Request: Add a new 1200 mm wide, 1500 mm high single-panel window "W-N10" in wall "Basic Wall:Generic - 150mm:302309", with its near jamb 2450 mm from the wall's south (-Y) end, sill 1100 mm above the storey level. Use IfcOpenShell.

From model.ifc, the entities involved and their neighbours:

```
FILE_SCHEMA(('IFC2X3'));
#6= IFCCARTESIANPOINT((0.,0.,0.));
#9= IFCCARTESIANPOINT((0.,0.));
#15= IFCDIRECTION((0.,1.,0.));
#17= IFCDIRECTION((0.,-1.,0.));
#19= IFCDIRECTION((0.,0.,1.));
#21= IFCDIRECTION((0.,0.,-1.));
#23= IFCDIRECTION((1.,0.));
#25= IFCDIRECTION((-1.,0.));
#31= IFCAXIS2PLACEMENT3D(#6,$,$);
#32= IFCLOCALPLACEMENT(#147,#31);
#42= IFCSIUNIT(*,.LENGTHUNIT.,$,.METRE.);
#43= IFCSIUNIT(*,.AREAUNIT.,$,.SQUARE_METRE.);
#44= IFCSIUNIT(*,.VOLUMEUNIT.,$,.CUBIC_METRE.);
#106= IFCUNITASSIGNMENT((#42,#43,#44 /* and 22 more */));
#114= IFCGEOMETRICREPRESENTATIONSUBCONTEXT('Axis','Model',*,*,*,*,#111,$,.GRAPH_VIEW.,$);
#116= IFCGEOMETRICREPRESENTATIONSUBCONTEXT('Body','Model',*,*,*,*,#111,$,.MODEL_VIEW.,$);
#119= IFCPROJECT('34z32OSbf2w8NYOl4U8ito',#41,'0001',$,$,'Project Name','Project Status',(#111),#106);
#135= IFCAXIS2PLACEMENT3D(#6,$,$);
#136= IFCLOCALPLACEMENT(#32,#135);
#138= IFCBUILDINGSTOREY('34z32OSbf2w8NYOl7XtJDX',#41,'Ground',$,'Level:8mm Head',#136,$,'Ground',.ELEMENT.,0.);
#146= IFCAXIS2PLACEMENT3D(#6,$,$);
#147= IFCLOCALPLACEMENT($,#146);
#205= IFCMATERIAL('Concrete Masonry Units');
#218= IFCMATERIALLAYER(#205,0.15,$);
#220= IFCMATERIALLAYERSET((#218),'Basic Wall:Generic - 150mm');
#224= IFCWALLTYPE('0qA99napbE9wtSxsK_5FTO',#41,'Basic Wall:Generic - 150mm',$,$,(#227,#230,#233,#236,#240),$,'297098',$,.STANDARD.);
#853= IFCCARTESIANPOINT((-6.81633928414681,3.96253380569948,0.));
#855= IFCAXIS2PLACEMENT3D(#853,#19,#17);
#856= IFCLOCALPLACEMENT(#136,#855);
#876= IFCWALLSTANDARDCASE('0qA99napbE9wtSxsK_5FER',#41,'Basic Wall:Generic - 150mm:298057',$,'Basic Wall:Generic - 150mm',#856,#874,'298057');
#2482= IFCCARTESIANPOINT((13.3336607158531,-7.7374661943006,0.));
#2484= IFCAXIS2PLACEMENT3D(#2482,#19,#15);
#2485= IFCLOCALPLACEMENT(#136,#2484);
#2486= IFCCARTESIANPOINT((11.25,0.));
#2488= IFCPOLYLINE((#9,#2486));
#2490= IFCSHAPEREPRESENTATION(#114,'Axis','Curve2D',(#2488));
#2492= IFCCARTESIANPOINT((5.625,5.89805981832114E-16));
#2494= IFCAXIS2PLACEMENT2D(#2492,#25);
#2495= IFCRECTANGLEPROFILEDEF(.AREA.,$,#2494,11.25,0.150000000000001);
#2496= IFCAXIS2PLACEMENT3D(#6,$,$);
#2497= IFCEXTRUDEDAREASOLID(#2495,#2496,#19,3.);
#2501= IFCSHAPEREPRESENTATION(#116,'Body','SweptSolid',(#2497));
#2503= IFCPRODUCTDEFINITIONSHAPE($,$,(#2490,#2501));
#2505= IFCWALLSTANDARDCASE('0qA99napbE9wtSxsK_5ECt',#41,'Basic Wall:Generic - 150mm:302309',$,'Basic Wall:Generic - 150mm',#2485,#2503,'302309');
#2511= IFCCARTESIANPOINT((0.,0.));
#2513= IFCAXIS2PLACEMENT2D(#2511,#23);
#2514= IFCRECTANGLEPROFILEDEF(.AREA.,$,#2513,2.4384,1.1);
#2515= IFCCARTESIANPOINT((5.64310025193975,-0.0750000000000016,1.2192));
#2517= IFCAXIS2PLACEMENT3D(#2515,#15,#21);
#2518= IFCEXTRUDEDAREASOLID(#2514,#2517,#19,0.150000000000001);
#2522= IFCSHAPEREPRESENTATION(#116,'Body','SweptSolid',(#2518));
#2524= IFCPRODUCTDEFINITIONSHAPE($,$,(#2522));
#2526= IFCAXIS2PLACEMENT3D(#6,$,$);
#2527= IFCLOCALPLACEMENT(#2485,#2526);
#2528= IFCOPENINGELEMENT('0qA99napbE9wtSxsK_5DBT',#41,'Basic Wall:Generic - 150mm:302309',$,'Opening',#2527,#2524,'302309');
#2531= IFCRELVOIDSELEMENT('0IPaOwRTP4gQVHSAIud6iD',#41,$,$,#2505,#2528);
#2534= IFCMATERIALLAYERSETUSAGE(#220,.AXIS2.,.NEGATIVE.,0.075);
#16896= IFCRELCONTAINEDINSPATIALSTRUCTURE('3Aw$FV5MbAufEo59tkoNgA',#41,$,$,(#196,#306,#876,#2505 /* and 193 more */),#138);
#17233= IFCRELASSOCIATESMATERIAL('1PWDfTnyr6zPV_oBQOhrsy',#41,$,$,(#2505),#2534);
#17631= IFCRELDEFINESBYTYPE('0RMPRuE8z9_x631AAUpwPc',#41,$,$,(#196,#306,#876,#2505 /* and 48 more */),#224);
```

```python
import numpy as np
import ifcopenshell
import ifcopenshell.api.feature
import ifcopenshell.api.geometry
import ifcopenshell.api.root
import ifcopenshell.api.spatial
import ifcopenshell.api.type
import ifcopenshell.geom
import ifcopenshell.util.element
import ifcopenshell.util.placement
import ifcopenshell.util.representation
import ifcopenshell.util.shape
import ifcopenshell.util.unit

model = ifcopenshell.open("model.ifc")
unit_scale = ifcopenshell.util.unit.calculate_unit_scale(model)
settings = ifcopenshell.geom.settings()


def volume(element):
    """Net volume in cubic metres, openings subtracted."""
    shape = ifcopenshell.geom.create_shape(settings, element)
    return ifcopenshell.util.shape.get_volume(shape.geometry)


wall = model.by_guid("0qA99napbE9wtSxsK_5ECt")
storey = ifcopenshell.util.element.get_container(wall, ifc_class="IfcBuildingStorey")
context = ifcopenshell.util.representation.get_context(model, "Model", "Body", "MODEL_VIEW")
before = volume(wall)

width, height, from_end, sill = 1.2, 1.5, 2.45, 1.1  # metres

# The wall runs along its own X axis, and the end named is its -X end.
wall_shape = ifcopenshell.geom.create_shape(settings, wall)
x, y, z = ifcopenshell.util.shape.get_vertices(wall_shape.geometry).T
start = x.min() + from_end
face, thickness = float(y.min()), float(y.max() - y.min())
wall_matrix = ifcopenshell.util.placement.get_local_placement(wall.ObjectPlacement)
level = ifcopenshell.util.placement.get_local_placement(storey.ObjectPlacement)[2, 3]


def in_wall(x, y):
    """Placement at x, y metres in the wall's axes, at sill height."""
    matrix = wall_matrix.copy()
    matrix[:, 3] = wall_matrix @ np.array([x / unit_scale, y / unit_scale, 0.0, 1.0])
    matrix[2, 3] = level + sill / unit_scale
    return matrix


# Opening: a box that overshoots both wall faces by 50 mm.
opening = ifcopenshell.api.root.create_entity(model, ifc_class="IfcOpeningElement")
box = ifcopenshell.api.geometry.add_wall_representation(
    model, context=context, length=width, height=height, thickness=thickness + 0.1
)
ifcopenshell.api.geometry.assign_representation(model, product=opening, representation=box)
ifcopenshell.api.geometry.edit_object_placement(model, product=opening, matrix=in_wall(start, face - 0.05), is_si=False)
ifcopenshell.api.feature.add_feature(model, feature=opening, element=wall)

window = ifcopenshell.api.root.create_entity(model, ifc_class="IfcWindow", name="W-N10")
window.OverallWidth, window.OverallHeight = width / unit_scale, height / unit_scale
body = ifcopenshell.api.geometry.add_window_representation(
    model,
    context=context,
    overall_width=window.OverallWidth,
    overall_height=window.OverallHeight,
    partition_type="SINGLE_PANEL",
)
ifcopenshell.api.geometry.assign_representation(model, product=window, representation=body)
ifcopenshell.api.spatial.assign_container(model, products=[window], relating_structure=storey)
fills = ifcopenshell.api.feature.add_filling(model, opening=opening, element=window)
fills.OwnerHistory = window.OwnerHistory  # required in IFC2X3

# IFC2X3 keeps the operation on the window style.
style = ifcopenshell.api.root.create_entity(model, ifc_class="IfcWindowStyle", name="W-N10")
style.OperationType, style.ConstructionType = "SINGLE_PANEL", "NOTDEFINED"
style.ParameterTakesPrecedence = style.Sizeable = False
ifcopenshell.api.type.assign_type(model, related_objects=[window], relating_type=style)

# Centre the window in the wall's thickness.
ifcopenshell.api.geometry.edit_object_placement(model, product=window, matrix=in_wall(start, face), is_si=False)
window_shape = ifcopenshell.geom.create_shape(settings, window)
depth = ifcopenshell.util.shape.get_vertices(window_shape.geometry)[:, 1]
offset = face + thickness / 2 - (depth.min() + depth.max()) / 2
ifcopenshell.api.geometry.edit_object_placement(model, product=window, matrix=in_wall(start, offset), is_si=False)

after = volume(wall)

print(f"wall volume {before:.3f} -> {after:.3f} m3")

model.write("model_edited.ifc")
```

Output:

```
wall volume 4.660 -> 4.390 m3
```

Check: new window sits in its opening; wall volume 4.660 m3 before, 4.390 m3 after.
